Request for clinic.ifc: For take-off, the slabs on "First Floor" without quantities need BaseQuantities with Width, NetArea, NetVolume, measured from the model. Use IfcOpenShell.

First a look at what the model holds.

```python
import ifcopenshell
import ifcopenshell.util.element
import ifcopenshell.util.unit

model = ifcopenshell.open("clinic.ifc")
print(model.schema)
for unit_type in ("LENGTHUNIT", "AREAUNIT", "VOLUMEUNIT"):
    print(unit_type, ifcopenshell.util.unit.calculate_unit_scale(model, unit_type))
storey = next(s for s in model.by_type("IfcBuildingStorey") if s.Name == "First Floor")
slabs = [e for e in ifcopenshell.util.element.get_decomposition(storey) if e.is_a("IfcSlab")]
for e in sorted(slabs, key=lambda e: e.id()):
    print(e.id(), e.is_a(), e.Name, list(ifcopenshell.util.element.get_psets(e, qtos_only=True)), sep=" | ")
```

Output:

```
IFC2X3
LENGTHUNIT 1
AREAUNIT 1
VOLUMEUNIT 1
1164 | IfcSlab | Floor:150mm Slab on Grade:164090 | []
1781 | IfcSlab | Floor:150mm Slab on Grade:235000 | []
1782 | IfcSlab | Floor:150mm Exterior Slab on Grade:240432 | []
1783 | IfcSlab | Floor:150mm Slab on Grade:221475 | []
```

```python
import ifcopenshell
import ifcopenshell.api.pset
import ifcopenshell.geom
import ifcopenshell.util.element
import ifcopenshell.util.shape
import ifcopenshell.util.unit

model = ifcopenshell.open("clinic.ifc")
unit_scale = ifcopenshell.util.unit.calculate_unit_scale(model)
area_scale = ifcopenshell.util.unit.calculate_unit_scale(model, "AREAUNIT")
volume_scale = ifcopenshell.util.unit.calculate_unit_scale(model, "VOLUMEUNIT")
settings = ifcopenshell.geom.settings()

storey = next(s for s in model.by_type("IfcBuildingStorey") if s.Name == "First Floor")
slabs = [e for e in ifcopenshell.util.element.get_decomposition(storey) if e.is_a("IfcSlab")]

for e in sorted(slabs, key=lambda e: e.id()):
    if ifcopenshell.util.element.get_psets(e, qtos_only=True, should_inherit=False):
        continue
    # Geometry comes back in metres, in the element's own axes.
    shape = ifcopenshell.geom.create_shape(settings, e)
    values = {
        "Width": ifcopenshell.util.shape.get_z(shape.geometry) / unit_scale,
        "NetArea": ifcopenshell.util.shape.get_footprint_area(shape.geometry) / area_scale,
        "NetVolume": ifcopenshell.util.shape.get_volume(shape.geometry) / volume_scale,
    }
    qto = ifcopenshell.api.pset.add_qto(model, product=e, name="BaseQuantities")
    ifcopenshell.api.pset.edit_qto(model, qto=qto, properties=values)
    print(e.id(), {k: round(v, 3) for k, v in values.items()})

model.write("clinic_rev.ifc")
```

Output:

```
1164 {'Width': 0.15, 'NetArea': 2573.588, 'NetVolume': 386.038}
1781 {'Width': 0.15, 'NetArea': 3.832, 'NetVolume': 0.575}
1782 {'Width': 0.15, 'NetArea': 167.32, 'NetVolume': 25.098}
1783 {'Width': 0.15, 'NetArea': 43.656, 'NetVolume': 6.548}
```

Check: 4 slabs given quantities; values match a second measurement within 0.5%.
